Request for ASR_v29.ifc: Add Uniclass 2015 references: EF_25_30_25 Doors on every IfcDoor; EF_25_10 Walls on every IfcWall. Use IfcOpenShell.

First a look at what the model holds.

```python
import ifcopenshell

model = ifcopenshell.open("ASR_v29.ifc")
print(model.schema)
print("classifications:", [c.Name for c in model.by_type("IfcClassification")])
for ifc_class in ("IfcDoor", "IfcRoof", "IfcStair", "IfcWall", "IfcWindow"):
    print(ifc_class, len(model.by_type(ifc_class)))
```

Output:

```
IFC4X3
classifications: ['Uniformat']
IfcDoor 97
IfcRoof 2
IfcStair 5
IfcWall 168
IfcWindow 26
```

```python
import ifcopenshell
import ifcopenshell.api.classification

model = ifcopenshell.open("ASR_v29.ifc")

system = ifcopenshell.api.classification.add_classification(model, classification="Uniclass 2015")

codes = {
    "IfcDoor": ("EF_25_30_25", "Doors"),
    "IfcWall": ("EF_25_10", "Walls"),
}
for ifc_class, (code, name) in codes.items():
    products = model.by_type(ifc_class)
    ifcopenshell.api.classification.add_reference(
        model, products=products, classification=system, identification=code, name=name
    )
    print(code, len(products))

model.write("ASR_v29_updated.ifc")
```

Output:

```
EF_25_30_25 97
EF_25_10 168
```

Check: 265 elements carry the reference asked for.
